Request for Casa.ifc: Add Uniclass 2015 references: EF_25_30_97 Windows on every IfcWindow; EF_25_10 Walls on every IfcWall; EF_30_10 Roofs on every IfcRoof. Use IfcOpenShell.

First a look at what the model holds.

```python
import ifcopenshell

model = ifcopenshell.open("Casa.ifc")
print(model.schema)
print("classifications:", [c.Name for c in model.by_type("IfcClassification")])
for ifc_class in ("IfcDoor", "IfcRoof", "IfcStair", "IfcWall", "IfcWindow"):
    print(ifc_class, len(model.by_type(ifc_class)))
```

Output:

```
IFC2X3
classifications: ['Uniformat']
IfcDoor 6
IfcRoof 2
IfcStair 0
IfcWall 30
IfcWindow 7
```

```python
import ifcopenshell
import ifcopenshell.api.classification

model = ifcopenshell.open("Casa.ifc")

# IFC2X3 requires Source and Edition and has no link from the project to the system.
system = model.create_entity("IfcClassification", Source="NBS", Edition="2015", Name="Uniclass 2015")

codes = {
    "IfcWindow": ("EF_25_30_97", "Windows"),
    "IfcWall": ("EF_25_10", "Walls"),
    "IfcRoof": ("EF_30_10", "Roofs"),
}
for ifc_class, (code, name) in codes.items():
    products = model.by_type(ifc_class)
    ifcopenshell.api.classification.add_reference(
        model, products=products, classification=system, identification=code, name=name
    )
    print(code, len(products))

model.write("Casa_edited.ifc")
```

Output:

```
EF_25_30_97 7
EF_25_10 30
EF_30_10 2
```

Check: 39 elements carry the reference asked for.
